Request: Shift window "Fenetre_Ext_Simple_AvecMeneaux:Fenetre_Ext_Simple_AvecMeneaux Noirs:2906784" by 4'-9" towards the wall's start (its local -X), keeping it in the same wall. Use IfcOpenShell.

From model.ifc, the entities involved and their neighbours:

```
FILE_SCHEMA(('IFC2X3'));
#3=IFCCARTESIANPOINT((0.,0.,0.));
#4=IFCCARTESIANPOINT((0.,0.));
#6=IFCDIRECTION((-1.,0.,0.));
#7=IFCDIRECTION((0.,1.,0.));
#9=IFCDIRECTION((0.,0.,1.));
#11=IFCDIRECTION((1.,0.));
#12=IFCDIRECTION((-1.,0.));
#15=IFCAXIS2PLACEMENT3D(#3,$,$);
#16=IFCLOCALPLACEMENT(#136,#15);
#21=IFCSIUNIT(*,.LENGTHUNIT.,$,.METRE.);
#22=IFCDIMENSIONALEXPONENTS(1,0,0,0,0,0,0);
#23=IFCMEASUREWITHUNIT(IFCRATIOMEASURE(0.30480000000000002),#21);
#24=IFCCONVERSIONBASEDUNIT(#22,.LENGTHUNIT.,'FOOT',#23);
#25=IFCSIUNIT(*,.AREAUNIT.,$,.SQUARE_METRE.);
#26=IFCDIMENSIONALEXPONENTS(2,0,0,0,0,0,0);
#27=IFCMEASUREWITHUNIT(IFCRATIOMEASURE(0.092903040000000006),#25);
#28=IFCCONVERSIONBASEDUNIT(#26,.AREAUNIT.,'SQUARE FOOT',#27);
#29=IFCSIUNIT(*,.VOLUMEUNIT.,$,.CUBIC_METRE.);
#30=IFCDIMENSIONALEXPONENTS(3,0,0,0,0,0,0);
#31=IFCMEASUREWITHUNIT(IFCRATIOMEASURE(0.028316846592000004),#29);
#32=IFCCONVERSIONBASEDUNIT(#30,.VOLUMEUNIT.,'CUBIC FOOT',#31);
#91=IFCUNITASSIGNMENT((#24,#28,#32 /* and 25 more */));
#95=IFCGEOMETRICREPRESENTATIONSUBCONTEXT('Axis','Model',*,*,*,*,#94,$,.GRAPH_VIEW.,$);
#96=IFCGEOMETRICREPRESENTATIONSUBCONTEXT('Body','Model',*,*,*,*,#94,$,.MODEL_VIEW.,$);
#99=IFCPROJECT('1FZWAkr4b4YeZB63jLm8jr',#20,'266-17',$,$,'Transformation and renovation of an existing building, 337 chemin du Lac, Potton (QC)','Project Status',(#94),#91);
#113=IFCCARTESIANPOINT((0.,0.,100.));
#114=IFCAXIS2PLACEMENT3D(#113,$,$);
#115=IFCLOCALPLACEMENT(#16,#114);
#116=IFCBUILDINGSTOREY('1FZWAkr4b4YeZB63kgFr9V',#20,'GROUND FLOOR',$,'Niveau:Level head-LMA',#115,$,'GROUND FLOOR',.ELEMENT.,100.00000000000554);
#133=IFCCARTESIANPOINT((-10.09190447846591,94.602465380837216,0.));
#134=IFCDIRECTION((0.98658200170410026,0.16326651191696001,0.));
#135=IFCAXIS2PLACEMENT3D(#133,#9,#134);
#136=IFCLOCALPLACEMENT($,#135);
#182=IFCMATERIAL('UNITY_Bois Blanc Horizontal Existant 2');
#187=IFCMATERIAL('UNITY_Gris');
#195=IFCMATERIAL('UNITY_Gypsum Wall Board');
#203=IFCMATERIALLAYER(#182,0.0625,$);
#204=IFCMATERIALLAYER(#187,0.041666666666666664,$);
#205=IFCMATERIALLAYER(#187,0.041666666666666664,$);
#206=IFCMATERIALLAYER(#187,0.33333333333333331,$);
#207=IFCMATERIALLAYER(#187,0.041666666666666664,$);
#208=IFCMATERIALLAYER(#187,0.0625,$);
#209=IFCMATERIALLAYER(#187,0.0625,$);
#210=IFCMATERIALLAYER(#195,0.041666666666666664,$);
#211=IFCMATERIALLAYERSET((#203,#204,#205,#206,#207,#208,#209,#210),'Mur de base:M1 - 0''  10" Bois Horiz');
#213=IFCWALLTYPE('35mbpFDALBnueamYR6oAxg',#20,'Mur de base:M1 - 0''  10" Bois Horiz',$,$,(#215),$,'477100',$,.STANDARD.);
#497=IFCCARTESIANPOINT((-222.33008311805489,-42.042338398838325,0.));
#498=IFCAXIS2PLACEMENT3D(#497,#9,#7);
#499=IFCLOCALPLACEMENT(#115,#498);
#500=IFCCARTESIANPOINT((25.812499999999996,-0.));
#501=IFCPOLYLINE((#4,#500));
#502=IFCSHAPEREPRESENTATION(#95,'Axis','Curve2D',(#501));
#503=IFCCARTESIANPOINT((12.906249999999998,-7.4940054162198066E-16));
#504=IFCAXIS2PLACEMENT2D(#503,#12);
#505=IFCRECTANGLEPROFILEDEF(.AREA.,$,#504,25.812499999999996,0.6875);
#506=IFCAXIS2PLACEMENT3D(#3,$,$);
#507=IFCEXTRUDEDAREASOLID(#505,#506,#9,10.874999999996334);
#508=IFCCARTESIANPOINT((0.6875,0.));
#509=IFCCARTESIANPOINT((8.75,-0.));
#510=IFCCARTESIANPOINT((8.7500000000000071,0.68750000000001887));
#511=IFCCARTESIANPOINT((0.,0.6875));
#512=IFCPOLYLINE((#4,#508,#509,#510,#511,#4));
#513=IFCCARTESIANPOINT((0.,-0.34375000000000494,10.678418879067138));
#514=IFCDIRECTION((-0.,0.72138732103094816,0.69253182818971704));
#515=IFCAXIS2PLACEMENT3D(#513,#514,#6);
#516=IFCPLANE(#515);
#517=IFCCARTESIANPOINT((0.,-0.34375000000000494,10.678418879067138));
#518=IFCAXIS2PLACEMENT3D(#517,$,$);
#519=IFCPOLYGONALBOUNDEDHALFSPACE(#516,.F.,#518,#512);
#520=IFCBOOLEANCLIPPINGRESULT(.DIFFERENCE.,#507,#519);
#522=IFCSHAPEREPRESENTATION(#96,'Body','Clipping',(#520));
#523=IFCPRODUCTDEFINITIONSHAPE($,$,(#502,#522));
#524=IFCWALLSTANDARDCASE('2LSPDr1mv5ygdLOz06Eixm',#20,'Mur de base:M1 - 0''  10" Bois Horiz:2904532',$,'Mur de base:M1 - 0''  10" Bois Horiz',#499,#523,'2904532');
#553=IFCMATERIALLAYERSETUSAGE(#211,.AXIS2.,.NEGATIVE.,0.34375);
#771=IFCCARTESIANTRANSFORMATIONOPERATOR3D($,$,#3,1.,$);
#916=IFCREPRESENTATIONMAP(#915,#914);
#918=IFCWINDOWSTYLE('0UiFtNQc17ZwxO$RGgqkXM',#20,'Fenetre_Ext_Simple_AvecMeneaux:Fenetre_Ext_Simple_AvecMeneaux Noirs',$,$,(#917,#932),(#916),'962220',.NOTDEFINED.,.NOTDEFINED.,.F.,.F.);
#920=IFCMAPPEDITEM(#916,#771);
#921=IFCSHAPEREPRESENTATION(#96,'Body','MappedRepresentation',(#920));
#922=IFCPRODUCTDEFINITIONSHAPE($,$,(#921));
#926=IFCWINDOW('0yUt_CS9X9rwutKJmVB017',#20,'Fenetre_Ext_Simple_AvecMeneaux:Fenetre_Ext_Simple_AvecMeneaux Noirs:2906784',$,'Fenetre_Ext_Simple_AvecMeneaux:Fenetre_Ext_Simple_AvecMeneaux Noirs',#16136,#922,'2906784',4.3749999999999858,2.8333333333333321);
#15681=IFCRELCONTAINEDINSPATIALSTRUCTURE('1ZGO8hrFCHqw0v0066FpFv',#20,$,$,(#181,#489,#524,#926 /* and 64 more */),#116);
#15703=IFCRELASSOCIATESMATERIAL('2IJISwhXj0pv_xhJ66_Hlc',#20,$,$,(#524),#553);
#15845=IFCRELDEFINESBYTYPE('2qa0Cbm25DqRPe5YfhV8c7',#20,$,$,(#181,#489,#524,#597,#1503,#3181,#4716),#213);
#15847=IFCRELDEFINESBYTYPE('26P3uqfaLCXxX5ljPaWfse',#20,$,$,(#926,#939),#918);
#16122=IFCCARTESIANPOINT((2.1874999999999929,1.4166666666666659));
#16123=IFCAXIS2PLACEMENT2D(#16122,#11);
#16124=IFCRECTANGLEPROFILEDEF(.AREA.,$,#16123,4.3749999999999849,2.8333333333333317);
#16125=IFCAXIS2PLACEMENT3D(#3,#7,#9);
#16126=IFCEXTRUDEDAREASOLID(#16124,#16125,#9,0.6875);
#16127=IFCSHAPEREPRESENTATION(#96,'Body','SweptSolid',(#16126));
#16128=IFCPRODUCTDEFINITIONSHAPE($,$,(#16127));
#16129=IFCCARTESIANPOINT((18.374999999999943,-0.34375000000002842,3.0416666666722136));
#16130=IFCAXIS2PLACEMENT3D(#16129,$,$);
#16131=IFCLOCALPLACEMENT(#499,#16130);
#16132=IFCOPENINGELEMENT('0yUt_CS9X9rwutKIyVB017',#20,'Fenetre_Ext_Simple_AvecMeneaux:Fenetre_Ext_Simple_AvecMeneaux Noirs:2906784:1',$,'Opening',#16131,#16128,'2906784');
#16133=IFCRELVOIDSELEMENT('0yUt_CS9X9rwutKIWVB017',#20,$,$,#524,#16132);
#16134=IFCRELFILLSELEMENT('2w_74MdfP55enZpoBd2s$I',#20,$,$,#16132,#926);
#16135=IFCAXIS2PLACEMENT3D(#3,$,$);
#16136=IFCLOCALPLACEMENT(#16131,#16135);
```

```python
import ifcopenshell
import ifcopenshell.api.geometry
import ifcopenshell.util.placement
import ifcopenshell.util.unit

model = ifcopenshell.open("model.ifc")
unit_scale = ifcopenshell.util.unit.calculate_unit_scale(model)

window = model.by_guid("0yUt_CS9X9rwutKJmVB017")
opening = window.FillsVoids[0].RelatingOpeningElement
wall = opening.VoidsElements[0].RelatingBuildingElement

wall_matrix = ifcopenshell.util.placement.get_local_placement(wall.ObjectPlacement)
shift = wall_matrix[:3, 0] * -57 * 0.0254 / unit_scale
before = ifcopenshell.util.placement.get_local_placement(window.ObjectPlacement)[:3, 3].copy()

# The window is placed relative to its opening, so it follows when the opening moves.
matrix = ifcopenshell.util.placement.get_local_placement(opening.ObjectPlacement)
matrix[:3, 3] += shift
ifcopenshell.api.geometry.edit_object_placement(
    model, product=opening, matrix=matrix, is_si=False, should_transform_children=True
)

after = ifcopenshell.util.placement.get_local_placement(window.ObjectPlacement)[:3, 3]
print("window moved by", (after - before).round(3) + 0.0)

model.write("model-out.ifc")
```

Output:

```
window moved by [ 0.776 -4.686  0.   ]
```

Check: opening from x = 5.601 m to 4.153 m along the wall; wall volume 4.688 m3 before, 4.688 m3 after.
